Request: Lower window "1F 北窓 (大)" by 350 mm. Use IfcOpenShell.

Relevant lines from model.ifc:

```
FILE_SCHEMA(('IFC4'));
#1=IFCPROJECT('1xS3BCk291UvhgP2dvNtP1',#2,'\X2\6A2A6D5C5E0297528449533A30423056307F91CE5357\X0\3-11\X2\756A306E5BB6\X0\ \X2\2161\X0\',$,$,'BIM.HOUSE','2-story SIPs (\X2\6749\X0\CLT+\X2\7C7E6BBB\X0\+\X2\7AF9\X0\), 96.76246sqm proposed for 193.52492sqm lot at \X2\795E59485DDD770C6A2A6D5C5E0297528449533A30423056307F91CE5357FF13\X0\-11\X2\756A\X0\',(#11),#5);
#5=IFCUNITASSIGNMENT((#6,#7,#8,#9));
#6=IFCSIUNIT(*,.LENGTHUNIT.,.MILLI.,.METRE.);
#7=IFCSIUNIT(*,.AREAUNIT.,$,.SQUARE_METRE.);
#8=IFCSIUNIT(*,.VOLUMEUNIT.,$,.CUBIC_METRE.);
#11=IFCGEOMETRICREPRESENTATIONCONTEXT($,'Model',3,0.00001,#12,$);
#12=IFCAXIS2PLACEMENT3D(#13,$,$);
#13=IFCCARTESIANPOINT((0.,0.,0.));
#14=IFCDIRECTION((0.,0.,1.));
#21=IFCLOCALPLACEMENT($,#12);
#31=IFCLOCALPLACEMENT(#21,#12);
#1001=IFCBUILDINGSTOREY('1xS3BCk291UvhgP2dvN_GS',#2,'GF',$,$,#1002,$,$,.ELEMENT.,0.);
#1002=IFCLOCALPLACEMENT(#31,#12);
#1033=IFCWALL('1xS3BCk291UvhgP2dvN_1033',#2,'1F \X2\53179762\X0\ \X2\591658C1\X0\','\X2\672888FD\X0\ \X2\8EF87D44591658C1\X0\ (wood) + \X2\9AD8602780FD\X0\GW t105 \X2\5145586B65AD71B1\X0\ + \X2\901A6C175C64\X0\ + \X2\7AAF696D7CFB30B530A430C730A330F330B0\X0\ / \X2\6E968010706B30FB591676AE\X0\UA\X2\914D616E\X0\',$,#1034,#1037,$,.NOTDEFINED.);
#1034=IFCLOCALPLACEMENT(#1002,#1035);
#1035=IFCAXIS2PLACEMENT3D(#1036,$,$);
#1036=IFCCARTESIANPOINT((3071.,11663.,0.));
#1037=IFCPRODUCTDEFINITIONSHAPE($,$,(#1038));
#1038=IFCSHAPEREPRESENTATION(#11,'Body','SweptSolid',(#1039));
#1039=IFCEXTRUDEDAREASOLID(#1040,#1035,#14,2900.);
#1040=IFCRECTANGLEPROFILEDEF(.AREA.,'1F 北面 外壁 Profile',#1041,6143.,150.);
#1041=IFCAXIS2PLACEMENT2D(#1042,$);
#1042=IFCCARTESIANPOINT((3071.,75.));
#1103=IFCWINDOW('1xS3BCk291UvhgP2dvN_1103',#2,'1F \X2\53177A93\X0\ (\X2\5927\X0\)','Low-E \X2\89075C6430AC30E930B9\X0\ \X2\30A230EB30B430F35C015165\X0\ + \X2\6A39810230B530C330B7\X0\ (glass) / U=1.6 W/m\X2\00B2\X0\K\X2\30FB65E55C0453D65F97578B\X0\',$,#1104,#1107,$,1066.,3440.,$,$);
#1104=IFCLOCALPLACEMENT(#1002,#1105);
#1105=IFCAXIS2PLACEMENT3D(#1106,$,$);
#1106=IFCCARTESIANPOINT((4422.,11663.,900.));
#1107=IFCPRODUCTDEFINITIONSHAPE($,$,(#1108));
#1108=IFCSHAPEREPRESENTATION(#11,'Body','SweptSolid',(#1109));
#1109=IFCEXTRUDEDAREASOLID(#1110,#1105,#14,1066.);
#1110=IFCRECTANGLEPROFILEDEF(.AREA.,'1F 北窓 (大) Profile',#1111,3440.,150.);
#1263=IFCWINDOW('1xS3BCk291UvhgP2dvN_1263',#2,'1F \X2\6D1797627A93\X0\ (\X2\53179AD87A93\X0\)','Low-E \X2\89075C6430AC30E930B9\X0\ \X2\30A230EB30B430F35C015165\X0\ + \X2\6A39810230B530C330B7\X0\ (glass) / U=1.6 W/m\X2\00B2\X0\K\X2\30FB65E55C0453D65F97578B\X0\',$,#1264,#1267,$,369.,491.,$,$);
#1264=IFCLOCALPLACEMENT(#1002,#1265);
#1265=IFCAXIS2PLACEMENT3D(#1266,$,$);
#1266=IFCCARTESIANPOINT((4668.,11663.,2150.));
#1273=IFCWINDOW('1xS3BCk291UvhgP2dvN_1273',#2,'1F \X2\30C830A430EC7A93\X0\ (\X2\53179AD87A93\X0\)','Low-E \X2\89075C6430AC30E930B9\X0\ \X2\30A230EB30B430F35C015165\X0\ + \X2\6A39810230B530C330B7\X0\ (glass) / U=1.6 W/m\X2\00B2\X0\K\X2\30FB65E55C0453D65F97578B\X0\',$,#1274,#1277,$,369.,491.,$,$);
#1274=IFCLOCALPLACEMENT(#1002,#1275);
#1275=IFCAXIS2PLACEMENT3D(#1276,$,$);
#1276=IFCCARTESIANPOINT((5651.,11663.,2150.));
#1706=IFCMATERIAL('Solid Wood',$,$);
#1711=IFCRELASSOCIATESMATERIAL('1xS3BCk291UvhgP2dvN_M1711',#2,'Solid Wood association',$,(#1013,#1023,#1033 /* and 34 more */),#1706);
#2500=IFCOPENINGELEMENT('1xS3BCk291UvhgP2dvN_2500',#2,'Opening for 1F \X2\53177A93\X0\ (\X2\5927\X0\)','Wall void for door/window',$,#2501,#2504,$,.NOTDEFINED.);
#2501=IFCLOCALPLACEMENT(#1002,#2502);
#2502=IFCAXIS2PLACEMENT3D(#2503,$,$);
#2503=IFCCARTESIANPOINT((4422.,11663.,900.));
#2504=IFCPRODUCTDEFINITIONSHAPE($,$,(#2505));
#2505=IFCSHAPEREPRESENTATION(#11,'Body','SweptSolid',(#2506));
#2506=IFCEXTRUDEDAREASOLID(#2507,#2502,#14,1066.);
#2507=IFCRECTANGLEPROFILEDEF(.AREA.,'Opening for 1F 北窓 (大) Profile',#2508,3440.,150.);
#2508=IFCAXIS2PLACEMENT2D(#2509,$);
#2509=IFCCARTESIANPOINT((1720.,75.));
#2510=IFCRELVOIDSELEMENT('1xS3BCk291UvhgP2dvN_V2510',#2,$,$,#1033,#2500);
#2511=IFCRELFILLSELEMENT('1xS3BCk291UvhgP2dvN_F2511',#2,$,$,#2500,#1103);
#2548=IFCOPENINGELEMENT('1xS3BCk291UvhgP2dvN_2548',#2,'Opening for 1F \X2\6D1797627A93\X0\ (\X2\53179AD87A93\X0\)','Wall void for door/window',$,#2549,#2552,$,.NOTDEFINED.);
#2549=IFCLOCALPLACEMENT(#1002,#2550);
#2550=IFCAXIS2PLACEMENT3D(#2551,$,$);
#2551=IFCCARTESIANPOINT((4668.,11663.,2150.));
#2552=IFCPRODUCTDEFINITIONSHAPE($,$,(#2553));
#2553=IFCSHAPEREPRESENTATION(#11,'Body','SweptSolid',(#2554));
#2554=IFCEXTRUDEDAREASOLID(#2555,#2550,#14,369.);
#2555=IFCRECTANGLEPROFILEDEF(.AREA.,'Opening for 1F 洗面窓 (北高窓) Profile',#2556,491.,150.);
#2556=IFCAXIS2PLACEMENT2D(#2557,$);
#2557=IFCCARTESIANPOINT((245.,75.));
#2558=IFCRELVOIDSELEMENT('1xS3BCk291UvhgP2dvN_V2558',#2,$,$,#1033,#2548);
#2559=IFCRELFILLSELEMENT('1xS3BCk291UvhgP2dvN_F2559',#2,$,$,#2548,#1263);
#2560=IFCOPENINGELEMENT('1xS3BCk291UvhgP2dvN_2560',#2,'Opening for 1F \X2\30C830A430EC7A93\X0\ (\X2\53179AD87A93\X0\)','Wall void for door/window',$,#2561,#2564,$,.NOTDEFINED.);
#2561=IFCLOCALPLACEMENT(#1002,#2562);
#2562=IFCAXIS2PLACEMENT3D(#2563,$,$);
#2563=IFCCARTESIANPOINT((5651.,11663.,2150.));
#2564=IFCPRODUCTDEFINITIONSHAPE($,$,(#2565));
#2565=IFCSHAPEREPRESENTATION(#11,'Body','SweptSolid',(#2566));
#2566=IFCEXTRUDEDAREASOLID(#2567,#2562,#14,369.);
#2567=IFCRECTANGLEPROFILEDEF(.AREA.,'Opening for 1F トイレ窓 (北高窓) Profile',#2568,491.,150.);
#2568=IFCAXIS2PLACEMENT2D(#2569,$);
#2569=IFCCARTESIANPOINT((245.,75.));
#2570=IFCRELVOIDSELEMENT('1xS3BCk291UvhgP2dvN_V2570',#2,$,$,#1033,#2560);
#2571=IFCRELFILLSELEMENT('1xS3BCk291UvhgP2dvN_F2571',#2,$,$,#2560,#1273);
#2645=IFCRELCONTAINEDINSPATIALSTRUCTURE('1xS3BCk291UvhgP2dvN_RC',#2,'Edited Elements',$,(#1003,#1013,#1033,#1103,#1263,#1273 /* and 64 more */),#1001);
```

```python
import numpy as np
import ifcopenshell
import ifcopenshell.api.geometry
import ifcopenshell.util.placement
import ifcopenshell.util.unit

model = ifcopenshell.open("model.ifc")
unit_scale = ifcopenshell.util.unit.calculate_unit_scale(model)

window = model.by_id(1103)
opening = window.FillsVoids[0].RelatingOpeningElement
dz = -350.0

shift = np.array([0.0, 0.0, dz])
# The window is not placed relative to its opening, so move both.
for product in (opening, window):
    matrix = ifcopenshell.util.placement.get_local_placement(product.ObjectPlacement)
    matrix[:3, 3] += shift
    ifcopenshell.api.geometry.edit_object_placement(model, product=product, matrix=matrix, is_si=False)

print(f"moved by {dz * unit_scale:+.3f} m")

model.write("model_v2.ifc")
```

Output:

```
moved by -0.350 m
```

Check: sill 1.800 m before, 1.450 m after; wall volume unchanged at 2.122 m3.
